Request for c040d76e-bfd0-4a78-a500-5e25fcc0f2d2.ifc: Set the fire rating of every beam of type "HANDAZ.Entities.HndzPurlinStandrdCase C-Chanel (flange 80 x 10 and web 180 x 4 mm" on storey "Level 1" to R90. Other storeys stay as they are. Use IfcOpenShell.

First a look at what the model holds.

```python
import ifcopenshell
import ifcopenshell.util.element

model = ifcopenshell.open("c040d76e-bfd0-4a78-a500-5e25fcc0f2d2.ifc")
print(model.schema)
storey = next(s for s in model.by_type("IfcBuildingStorey") if s.Name == "Level 1")
beams = [e for e in ifcopenshell.util.element.get_decomposition(storey) if e.is_a("IfcBeam")]
seen = {}
for e in beams:
    element_type = ifcopenshell.util.element.get_type(e)
    key = (element_type.Name if element_type != e and element_type else None, ifcopenshell.util.element.get_pset(e, "Pset_BeamCommon", "FireRating"))
    seen[key] = seen.get(key, 0) + 1
for (name, value), count in sorted(seen.items(), key=str):
    print(count, "x", name, "|", value)
```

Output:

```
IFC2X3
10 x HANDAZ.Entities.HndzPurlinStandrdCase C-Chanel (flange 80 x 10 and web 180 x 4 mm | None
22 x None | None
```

```python
import ifcopenshell
import ifcopenshell.api.pset
import ifcopenshell.util.element

model = ifcopenshell.open("c040d76e-bfd0-4a78-a500-5e25fcc0f2d2.ifc")

storey = next(s for s in model.by_type("IfcBuildingStorey") if s.Name == "Level 1")
beams = [e for e in ifcopenshell.util.element.get_decomposition(storey) if e.is_a("IfcBeam")]

count = 0
for e in beams:
    element_type = ifcopenshell.util.element.get_type(e)
    if element_type in (None, e) or element_type.Name != "HANDAZ.Entities.HndzPurlinStandrdCase C-Chanel (flange 80 x 10 and web 180 x 4 mm":
        continue
    # add_pset returns the element's existing set when there is one.
    pset = ifcopenshell.api.pset.add_pset(model, product=e, name="Pset_BeamCommon")
    ifcopenshell.api.pset.edit_pset(model, pset=pset, properties={"FireRating": "R90"})
    count += 1

print(count, "beams updated")

model.write("c040d76e-bfd0-4a78-a500-5e25fcc0f2d2_rev.ifc")
```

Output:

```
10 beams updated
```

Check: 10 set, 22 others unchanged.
